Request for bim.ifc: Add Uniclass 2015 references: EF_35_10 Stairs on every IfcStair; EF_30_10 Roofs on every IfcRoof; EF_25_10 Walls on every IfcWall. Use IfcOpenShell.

First a look at what the model holds.

```python
import ifcopenshell

model = ifcopenshell.open("bim.ifc")
print(model.schema)
print("classifications:", [c.Name for c in model.by_type("IfcClassification")])
for ifc_class in ("IfcDoor", "IfcRoof", "IfcStair", "IfcWall", "IfcWindow"):
    print(ifc_class, len(model.by_type(ifc_class)))
```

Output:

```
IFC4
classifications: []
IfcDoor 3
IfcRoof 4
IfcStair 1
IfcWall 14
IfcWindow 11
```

```python
import ifcopenshell
import ifcopenshell.api.classification

model = ifcopenshell.open("bim.ifc")

system = ifcopenshell.api.classification.add_classification(model, classification="Uniclass 2015")

codes = {
    "IfcStair": ("EF_35_10", "Stairs"),
    "IfcRoof": ("EF_30_10", "Roofs"),
    "IfcWall": ("EF_25_10", "Walls"),
}
for ifc_class, (code, name) in codes.items():
    products = model.by_type(ifc_class)
    ifcopenshell.api.classification.add_reference(
        model, products=products, classification=system, identification=code, name=name
    )
    print(code, len(products))

model.write("bim_updated.ifc")
```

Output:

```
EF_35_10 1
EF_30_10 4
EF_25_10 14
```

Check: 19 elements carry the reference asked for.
